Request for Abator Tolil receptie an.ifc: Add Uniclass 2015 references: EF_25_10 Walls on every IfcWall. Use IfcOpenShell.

First a look at what the model holds.

```python
import ifcopenshell

model = ifcopenshell.open("Abator Tolil receptie an.ifc")
print(model.schema)
print("classifications:", [c.Name for c in model.by_type("IfcClassification")])
for ifc_class in ("IfcDoor", "IfcRoof", "IfcStair", "IfcWall", "IfcWindow"):
    print(ifc_class, len(model.by_type(ifc_class)))
```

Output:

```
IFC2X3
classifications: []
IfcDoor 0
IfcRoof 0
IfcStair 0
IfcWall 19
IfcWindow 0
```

```python
import ifcopenshell
import ifcopenshell.api.classification

model = ifcopenshell.open("Abator Tolil receptie an.ifc")

# IFC2X3 requires Source and Edition and has no link from the project to the system.
system = model.create_entity("IfcClassification", Source="NBS", Edition="2015", Name="Uniclass 2015")

codes = {
    "IfcWall": ("EF_25_10", "Walls"),
}
for ifc_class, (code, name) in codes.items():
    products = model.by_type(ifc_class)
    ifcopenshell.api.classification.add_reference(
        model, products=products, classification=system, identification=code, name=name
    )
    print(code, len(products))

model.write("Abator Tolil receptie an_edited.ifc")
```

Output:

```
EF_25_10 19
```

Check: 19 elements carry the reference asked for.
